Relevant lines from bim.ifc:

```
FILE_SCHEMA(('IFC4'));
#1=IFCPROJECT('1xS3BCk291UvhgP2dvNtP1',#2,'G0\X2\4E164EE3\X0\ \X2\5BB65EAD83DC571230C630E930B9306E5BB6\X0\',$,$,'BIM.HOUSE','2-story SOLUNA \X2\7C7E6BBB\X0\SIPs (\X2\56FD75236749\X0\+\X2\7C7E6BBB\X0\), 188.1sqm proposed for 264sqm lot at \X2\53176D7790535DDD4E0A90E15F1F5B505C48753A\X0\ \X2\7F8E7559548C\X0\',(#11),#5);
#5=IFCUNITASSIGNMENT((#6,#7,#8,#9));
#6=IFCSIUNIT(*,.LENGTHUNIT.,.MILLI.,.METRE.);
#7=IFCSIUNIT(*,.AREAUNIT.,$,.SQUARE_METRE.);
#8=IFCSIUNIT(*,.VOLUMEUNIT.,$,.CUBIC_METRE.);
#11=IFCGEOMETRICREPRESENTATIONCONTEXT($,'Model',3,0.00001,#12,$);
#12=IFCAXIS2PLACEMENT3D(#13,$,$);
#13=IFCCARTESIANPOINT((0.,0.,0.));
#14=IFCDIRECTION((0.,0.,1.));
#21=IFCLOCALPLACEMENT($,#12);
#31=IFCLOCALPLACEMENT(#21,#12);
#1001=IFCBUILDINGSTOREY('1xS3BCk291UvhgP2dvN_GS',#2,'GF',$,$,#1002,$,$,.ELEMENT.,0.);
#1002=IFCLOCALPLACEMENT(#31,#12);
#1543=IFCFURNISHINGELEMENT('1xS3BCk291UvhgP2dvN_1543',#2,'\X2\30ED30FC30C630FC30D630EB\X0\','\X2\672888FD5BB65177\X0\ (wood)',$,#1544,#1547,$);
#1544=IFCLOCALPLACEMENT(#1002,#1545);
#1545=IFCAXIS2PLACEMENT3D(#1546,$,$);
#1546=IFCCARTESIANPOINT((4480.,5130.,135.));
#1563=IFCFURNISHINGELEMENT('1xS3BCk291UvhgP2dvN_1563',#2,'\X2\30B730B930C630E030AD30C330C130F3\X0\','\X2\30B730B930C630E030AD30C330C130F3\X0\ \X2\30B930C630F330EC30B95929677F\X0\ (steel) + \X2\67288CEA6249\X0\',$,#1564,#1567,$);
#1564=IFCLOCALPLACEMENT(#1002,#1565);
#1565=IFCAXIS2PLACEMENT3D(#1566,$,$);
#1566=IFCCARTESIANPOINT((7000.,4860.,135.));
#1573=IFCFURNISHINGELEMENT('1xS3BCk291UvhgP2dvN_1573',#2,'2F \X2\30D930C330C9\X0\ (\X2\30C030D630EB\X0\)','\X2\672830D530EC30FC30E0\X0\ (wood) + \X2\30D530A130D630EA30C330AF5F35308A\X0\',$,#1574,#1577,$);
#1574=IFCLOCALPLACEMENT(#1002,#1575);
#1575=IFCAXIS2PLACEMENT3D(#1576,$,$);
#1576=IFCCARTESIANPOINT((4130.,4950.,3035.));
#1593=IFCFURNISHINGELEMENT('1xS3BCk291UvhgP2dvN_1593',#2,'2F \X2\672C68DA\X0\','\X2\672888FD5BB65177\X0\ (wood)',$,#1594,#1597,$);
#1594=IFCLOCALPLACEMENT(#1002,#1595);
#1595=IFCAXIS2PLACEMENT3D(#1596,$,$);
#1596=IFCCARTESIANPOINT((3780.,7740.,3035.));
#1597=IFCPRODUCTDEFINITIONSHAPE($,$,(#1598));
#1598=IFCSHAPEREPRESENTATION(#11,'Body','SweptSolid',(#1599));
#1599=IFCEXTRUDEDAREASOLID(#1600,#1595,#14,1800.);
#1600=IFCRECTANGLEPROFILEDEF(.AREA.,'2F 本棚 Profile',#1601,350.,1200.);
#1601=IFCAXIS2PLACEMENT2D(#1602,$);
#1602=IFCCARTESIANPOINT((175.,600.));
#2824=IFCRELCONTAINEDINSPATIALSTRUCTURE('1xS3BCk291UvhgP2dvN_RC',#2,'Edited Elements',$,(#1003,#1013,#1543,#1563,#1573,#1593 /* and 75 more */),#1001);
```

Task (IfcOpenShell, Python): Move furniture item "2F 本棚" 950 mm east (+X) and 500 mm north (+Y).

```python
import ifcopenshell
import ifcopenshell.api.geometry
import ifcopenshell.util.placement

model = ifcopenshell.open("bim.ifc")

item = model.by_guid("1xS3BCk291UvhgP2dvN_1593")
matrix = ifcopenshell.util.placement.get_local_placement(item.ObjectPlacement)
matrix[0, 3] += 950.0
matrix[1, 3] += 500.0
ifcopenshell.api.geometry.edit_object_placement(model, product=item, matrix=matrix, is_si=False)

print(ifcopenshell.util.placement.get_local_placement(item.ObjectPlacement).round(3) + 0.0)

model.write("bim_rev.ifc")
```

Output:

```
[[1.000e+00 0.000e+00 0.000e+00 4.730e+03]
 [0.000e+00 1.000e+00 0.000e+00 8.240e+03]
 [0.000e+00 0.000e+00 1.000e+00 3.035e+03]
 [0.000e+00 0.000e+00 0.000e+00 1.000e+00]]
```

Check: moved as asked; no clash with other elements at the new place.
